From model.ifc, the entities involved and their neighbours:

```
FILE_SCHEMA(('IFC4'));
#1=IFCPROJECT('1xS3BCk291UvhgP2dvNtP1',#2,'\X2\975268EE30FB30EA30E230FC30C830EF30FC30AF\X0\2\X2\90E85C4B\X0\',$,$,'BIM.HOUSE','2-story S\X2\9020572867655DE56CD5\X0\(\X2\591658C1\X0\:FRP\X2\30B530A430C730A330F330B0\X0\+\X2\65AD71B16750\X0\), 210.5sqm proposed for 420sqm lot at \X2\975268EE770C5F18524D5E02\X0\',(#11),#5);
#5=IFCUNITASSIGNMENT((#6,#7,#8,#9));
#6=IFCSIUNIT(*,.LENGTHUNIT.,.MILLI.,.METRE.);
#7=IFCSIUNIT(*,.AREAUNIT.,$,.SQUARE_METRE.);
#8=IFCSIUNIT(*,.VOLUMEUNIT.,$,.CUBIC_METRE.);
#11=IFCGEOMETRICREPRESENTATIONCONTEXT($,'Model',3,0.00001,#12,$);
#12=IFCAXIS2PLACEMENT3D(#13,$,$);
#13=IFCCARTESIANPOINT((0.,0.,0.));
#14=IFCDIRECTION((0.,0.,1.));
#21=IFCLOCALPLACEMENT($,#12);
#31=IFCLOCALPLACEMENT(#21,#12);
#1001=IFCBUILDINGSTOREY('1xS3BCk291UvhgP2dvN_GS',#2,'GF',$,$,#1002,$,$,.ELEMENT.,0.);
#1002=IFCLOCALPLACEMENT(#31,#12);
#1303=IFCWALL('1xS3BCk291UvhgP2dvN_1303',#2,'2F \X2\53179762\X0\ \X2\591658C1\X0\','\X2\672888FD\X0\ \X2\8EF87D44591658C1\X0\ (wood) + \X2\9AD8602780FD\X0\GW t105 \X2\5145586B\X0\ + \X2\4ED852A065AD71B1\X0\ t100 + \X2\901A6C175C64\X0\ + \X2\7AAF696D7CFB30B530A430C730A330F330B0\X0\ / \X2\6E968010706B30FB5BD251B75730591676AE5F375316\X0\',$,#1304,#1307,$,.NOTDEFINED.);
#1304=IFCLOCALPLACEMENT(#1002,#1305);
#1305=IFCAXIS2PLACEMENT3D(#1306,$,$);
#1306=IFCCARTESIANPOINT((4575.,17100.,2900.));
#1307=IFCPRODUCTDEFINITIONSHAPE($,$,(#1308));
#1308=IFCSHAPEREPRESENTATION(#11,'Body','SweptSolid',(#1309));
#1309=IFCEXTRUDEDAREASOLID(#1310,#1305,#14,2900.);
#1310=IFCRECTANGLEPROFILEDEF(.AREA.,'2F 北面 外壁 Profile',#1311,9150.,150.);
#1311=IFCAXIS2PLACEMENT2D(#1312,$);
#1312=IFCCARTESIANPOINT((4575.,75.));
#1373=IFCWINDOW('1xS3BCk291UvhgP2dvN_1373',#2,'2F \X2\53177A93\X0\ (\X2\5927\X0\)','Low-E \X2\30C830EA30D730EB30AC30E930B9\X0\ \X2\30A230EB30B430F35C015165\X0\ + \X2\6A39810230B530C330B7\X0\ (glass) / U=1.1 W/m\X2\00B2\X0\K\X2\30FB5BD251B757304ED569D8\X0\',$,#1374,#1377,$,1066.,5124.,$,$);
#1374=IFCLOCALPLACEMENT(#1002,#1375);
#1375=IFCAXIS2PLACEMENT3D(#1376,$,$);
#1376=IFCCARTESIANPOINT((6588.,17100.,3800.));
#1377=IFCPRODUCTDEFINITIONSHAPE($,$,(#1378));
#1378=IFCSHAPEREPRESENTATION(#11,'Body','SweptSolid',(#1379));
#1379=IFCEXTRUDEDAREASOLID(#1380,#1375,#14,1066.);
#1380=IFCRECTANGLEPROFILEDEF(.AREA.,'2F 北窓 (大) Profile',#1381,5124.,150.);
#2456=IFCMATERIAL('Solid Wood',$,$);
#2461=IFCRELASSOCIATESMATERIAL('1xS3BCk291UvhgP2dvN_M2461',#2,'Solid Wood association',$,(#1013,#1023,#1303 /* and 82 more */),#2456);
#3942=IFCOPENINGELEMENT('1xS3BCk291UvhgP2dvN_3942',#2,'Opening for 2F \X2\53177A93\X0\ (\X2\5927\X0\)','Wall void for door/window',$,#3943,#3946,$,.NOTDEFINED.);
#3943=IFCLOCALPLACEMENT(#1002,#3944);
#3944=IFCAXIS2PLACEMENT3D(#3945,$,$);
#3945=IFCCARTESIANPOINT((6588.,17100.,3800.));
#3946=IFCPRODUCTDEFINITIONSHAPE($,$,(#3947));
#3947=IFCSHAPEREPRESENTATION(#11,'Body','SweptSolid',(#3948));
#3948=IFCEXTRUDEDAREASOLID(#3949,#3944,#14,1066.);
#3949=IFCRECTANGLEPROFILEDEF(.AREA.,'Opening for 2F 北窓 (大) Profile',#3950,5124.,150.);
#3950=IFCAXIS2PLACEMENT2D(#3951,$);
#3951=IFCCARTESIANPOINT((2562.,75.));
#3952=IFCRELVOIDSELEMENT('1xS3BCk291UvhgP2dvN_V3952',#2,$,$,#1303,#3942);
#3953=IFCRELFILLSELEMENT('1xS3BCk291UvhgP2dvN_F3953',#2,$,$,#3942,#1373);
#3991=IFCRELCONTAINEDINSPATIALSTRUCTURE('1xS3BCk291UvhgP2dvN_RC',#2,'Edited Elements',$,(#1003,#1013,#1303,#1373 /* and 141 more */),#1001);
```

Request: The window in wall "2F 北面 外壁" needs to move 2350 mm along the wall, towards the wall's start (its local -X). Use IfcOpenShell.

```python
import ifcopenshell
import ifcopenshell.api.geometry
import ifcopenshell.util.placement

model = ifcopenshell.open("model.ifc")

window = model.by_guid("1xS3BCk291UvhgP2dvN_1373")
opening = window.FillsVoids[0].RelatingOpeningElement
wall = opening.VoidsElements[0].RelatingBuildingElement

wall_matrix = ifcopenshell.util.placement.get_local_placement(wall.ObjectPlacement)
shift = wall_matrix[:3, 0] * -2350.0
before = ifcopenshell.util.placement.get_local_placement(window.ObjectPlacement)[:3, 3].copy()

# The window is not placed relative to its opening, so move both.
for product in (opening, window):
    matrix = ifcopenshell.util.placement.get_local_placement(product.ObjectPlacement)
    matrix[:3, 3] += shift
    ifcopenshell.api.geometry.edit_object_placement(model, product=product, matrix=matrix, is_si=False)

after = ifcopenshell.util.placement.get_local_placement(window.ObjectPlacement)[:3, 3]
print("window moved by", (after - before).round(3) + 0.0)

model.write("model_edited.ifc")
```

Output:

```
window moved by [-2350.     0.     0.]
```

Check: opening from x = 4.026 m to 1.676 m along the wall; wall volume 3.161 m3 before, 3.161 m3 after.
